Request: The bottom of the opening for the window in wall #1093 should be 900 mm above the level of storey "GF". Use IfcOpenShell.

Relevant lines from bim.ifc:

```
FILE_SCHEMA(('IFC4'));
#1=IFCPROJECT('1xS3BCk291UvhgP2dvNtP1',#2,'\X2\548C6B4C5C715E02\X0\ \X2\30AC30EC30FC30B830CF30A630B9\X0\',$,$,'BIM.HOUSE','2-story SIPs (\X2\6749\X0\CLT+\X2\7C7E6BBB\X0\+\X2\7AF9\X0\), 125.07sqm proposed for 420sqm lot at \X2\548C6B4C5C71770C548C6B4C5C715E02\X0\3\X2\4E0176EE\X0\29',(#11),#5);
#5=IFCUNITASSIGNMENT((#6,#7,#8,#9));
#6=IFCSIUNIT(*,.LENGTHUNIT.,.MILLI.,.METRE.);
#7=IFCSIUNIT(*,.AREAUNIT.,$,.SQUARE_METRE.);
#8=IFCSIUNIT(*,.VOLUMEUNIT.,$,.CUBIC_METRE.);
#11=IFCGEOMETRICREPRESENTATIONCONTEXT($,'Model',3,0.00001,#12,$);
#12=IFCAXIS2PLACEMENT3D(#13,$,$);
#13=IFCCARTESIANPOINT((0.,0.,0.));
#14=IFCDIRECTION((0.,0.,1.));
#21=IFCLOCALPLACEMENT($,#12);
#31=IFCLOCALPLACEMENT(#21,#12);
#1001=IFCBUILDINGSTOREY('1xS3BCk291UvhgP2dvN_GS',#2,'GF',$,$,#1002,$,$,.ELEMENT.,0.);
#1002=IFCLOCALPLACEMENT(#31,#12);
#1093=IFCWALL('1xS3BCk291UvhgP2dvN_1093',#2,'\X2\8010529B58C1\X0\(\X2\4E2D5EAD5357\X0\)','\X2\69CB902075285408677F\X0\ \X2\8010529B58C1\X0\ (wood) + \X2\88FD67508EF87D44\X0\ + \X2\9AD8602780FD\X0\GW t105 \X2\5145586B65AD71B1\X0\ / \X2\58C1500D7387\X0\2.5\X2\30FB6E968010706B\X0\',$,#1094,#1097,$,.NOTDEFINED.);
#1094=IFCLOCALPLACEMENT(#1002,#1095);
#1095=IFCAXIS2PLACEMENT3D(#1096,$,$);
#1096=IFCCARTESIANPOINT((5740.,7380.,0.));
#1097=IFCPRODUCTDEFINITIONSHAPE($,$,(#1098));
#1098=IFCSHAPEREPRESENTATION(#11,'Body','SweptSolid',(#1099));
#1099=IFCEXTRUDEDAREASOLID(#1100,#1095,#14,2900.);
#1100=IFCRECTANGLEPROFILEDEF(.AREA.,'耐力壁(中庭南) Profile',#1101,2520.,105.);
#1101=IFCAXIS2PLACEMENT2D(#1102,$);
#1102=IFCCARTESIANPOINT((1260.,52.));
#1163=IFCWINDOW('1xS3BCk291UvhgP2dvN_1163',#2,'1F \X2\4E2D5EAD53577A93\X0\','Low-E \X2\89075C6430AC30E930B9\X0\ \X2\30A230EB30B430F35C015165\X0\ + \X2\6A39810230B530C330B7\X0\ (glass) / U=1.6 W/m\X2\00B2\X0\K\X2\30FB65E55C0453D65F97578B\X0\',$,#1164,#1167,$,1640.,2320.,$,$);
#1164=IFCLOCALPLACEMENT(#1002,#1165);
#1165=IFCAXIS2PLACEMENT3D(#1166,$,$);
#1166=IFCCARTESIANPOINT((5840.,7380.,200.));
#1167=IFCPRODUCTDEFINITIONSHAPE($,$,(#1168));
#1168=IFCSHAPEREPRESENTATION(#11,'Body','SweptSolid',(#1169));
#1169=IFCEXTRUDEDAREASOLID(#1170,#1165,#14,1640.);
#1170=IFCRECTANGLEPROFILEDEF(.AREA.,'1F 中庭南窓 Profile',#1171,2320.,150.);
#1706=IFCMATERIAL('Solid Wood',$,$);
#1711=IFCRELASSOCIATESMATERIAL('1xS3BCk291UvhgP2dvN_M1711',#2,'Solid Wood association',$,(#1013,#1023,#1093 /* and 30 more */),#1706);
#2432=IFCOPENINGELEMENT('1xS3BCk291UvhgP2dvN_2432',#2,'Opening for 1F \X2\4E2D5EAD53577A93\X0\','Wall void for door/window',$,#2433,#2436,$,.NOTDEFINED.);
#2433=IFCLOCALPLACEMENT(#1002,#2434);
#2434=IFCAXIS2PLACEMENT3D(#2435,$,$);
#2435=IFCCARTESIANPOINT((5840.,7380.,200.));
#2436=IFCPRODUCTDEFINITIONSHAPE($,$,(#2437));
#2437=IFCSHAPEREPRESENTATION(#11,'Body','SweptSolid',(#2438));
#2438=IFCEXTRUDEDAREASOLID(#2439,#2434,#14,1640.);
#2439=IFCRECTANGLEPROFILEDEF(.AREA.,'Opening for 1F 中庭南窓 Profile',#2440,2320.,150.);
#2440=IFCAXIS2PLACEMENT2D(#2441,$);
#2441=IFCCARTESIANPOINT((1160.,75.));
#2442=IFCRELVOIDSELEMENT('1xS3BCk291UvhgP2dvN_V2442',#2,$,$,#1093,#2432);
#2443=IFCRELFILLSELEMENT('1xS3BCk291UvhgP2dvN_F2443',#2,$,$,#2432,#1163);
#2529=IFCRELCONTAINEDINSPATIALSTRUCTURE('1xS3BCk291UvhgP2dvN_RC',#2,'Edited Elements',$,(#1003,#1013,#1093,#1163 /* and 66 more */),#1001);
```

```python
import numpy as np
import ifcopenshell
import ifcopenshell.api.geometry
import ifcopenshell.geom
import ifcopenshell.util.element
import ifcopenshell.util.placement
import ifcopenshell.util.shape
import ifcopenshell.util.unit

model = ifcopenshell.open("bim.ifc")
unit_scale = ifcopenshell.util.unit.calculate_unit_scale(model)

window = model.by_guid("1xS3BCk291UvhgP2dvN_1163")
opening = window.FillsVoids[0].RelatingOpeningElement
storey = ifcopenshell.util.element.get_container(window, ifc_class="IfcBuildingStorey")
level = ifcopenshell.util.placement.get_local_placement(storey.ObjectPlacement)[2, 3]

# The opening's origin need not be at the sill, so measure its lowest point.
shape = ifcopenshell.geom.create_shape(ifcopenshell.geom.settings(), opening)
bottom = ifcopenshell.util.shape.get_shape_bottom_elevation(shape, shape.geometry) / unit_scale
dz = level + 0.9 / unit_scale - bottom

shift = np.array([0.0, 0.0, dz])
# The window is not placed relative to its opening, so move both.
for product in (opening, window):
    matrix = ifcopenshell.util.placement.get_local_placement(product.ObjectPlacement)
    matrix[:3, 3] += shift
    ifcopenshell.api.geometry.edit_object_placement(model, product=product, matrix=matrix, is_si=False)

print(f"moved by {dz * unit_scale:+.3f} m")

model.write("bim-out.ifc")
```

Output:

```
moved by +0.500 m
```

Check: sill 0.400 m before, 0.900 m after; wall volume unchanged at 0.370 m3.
